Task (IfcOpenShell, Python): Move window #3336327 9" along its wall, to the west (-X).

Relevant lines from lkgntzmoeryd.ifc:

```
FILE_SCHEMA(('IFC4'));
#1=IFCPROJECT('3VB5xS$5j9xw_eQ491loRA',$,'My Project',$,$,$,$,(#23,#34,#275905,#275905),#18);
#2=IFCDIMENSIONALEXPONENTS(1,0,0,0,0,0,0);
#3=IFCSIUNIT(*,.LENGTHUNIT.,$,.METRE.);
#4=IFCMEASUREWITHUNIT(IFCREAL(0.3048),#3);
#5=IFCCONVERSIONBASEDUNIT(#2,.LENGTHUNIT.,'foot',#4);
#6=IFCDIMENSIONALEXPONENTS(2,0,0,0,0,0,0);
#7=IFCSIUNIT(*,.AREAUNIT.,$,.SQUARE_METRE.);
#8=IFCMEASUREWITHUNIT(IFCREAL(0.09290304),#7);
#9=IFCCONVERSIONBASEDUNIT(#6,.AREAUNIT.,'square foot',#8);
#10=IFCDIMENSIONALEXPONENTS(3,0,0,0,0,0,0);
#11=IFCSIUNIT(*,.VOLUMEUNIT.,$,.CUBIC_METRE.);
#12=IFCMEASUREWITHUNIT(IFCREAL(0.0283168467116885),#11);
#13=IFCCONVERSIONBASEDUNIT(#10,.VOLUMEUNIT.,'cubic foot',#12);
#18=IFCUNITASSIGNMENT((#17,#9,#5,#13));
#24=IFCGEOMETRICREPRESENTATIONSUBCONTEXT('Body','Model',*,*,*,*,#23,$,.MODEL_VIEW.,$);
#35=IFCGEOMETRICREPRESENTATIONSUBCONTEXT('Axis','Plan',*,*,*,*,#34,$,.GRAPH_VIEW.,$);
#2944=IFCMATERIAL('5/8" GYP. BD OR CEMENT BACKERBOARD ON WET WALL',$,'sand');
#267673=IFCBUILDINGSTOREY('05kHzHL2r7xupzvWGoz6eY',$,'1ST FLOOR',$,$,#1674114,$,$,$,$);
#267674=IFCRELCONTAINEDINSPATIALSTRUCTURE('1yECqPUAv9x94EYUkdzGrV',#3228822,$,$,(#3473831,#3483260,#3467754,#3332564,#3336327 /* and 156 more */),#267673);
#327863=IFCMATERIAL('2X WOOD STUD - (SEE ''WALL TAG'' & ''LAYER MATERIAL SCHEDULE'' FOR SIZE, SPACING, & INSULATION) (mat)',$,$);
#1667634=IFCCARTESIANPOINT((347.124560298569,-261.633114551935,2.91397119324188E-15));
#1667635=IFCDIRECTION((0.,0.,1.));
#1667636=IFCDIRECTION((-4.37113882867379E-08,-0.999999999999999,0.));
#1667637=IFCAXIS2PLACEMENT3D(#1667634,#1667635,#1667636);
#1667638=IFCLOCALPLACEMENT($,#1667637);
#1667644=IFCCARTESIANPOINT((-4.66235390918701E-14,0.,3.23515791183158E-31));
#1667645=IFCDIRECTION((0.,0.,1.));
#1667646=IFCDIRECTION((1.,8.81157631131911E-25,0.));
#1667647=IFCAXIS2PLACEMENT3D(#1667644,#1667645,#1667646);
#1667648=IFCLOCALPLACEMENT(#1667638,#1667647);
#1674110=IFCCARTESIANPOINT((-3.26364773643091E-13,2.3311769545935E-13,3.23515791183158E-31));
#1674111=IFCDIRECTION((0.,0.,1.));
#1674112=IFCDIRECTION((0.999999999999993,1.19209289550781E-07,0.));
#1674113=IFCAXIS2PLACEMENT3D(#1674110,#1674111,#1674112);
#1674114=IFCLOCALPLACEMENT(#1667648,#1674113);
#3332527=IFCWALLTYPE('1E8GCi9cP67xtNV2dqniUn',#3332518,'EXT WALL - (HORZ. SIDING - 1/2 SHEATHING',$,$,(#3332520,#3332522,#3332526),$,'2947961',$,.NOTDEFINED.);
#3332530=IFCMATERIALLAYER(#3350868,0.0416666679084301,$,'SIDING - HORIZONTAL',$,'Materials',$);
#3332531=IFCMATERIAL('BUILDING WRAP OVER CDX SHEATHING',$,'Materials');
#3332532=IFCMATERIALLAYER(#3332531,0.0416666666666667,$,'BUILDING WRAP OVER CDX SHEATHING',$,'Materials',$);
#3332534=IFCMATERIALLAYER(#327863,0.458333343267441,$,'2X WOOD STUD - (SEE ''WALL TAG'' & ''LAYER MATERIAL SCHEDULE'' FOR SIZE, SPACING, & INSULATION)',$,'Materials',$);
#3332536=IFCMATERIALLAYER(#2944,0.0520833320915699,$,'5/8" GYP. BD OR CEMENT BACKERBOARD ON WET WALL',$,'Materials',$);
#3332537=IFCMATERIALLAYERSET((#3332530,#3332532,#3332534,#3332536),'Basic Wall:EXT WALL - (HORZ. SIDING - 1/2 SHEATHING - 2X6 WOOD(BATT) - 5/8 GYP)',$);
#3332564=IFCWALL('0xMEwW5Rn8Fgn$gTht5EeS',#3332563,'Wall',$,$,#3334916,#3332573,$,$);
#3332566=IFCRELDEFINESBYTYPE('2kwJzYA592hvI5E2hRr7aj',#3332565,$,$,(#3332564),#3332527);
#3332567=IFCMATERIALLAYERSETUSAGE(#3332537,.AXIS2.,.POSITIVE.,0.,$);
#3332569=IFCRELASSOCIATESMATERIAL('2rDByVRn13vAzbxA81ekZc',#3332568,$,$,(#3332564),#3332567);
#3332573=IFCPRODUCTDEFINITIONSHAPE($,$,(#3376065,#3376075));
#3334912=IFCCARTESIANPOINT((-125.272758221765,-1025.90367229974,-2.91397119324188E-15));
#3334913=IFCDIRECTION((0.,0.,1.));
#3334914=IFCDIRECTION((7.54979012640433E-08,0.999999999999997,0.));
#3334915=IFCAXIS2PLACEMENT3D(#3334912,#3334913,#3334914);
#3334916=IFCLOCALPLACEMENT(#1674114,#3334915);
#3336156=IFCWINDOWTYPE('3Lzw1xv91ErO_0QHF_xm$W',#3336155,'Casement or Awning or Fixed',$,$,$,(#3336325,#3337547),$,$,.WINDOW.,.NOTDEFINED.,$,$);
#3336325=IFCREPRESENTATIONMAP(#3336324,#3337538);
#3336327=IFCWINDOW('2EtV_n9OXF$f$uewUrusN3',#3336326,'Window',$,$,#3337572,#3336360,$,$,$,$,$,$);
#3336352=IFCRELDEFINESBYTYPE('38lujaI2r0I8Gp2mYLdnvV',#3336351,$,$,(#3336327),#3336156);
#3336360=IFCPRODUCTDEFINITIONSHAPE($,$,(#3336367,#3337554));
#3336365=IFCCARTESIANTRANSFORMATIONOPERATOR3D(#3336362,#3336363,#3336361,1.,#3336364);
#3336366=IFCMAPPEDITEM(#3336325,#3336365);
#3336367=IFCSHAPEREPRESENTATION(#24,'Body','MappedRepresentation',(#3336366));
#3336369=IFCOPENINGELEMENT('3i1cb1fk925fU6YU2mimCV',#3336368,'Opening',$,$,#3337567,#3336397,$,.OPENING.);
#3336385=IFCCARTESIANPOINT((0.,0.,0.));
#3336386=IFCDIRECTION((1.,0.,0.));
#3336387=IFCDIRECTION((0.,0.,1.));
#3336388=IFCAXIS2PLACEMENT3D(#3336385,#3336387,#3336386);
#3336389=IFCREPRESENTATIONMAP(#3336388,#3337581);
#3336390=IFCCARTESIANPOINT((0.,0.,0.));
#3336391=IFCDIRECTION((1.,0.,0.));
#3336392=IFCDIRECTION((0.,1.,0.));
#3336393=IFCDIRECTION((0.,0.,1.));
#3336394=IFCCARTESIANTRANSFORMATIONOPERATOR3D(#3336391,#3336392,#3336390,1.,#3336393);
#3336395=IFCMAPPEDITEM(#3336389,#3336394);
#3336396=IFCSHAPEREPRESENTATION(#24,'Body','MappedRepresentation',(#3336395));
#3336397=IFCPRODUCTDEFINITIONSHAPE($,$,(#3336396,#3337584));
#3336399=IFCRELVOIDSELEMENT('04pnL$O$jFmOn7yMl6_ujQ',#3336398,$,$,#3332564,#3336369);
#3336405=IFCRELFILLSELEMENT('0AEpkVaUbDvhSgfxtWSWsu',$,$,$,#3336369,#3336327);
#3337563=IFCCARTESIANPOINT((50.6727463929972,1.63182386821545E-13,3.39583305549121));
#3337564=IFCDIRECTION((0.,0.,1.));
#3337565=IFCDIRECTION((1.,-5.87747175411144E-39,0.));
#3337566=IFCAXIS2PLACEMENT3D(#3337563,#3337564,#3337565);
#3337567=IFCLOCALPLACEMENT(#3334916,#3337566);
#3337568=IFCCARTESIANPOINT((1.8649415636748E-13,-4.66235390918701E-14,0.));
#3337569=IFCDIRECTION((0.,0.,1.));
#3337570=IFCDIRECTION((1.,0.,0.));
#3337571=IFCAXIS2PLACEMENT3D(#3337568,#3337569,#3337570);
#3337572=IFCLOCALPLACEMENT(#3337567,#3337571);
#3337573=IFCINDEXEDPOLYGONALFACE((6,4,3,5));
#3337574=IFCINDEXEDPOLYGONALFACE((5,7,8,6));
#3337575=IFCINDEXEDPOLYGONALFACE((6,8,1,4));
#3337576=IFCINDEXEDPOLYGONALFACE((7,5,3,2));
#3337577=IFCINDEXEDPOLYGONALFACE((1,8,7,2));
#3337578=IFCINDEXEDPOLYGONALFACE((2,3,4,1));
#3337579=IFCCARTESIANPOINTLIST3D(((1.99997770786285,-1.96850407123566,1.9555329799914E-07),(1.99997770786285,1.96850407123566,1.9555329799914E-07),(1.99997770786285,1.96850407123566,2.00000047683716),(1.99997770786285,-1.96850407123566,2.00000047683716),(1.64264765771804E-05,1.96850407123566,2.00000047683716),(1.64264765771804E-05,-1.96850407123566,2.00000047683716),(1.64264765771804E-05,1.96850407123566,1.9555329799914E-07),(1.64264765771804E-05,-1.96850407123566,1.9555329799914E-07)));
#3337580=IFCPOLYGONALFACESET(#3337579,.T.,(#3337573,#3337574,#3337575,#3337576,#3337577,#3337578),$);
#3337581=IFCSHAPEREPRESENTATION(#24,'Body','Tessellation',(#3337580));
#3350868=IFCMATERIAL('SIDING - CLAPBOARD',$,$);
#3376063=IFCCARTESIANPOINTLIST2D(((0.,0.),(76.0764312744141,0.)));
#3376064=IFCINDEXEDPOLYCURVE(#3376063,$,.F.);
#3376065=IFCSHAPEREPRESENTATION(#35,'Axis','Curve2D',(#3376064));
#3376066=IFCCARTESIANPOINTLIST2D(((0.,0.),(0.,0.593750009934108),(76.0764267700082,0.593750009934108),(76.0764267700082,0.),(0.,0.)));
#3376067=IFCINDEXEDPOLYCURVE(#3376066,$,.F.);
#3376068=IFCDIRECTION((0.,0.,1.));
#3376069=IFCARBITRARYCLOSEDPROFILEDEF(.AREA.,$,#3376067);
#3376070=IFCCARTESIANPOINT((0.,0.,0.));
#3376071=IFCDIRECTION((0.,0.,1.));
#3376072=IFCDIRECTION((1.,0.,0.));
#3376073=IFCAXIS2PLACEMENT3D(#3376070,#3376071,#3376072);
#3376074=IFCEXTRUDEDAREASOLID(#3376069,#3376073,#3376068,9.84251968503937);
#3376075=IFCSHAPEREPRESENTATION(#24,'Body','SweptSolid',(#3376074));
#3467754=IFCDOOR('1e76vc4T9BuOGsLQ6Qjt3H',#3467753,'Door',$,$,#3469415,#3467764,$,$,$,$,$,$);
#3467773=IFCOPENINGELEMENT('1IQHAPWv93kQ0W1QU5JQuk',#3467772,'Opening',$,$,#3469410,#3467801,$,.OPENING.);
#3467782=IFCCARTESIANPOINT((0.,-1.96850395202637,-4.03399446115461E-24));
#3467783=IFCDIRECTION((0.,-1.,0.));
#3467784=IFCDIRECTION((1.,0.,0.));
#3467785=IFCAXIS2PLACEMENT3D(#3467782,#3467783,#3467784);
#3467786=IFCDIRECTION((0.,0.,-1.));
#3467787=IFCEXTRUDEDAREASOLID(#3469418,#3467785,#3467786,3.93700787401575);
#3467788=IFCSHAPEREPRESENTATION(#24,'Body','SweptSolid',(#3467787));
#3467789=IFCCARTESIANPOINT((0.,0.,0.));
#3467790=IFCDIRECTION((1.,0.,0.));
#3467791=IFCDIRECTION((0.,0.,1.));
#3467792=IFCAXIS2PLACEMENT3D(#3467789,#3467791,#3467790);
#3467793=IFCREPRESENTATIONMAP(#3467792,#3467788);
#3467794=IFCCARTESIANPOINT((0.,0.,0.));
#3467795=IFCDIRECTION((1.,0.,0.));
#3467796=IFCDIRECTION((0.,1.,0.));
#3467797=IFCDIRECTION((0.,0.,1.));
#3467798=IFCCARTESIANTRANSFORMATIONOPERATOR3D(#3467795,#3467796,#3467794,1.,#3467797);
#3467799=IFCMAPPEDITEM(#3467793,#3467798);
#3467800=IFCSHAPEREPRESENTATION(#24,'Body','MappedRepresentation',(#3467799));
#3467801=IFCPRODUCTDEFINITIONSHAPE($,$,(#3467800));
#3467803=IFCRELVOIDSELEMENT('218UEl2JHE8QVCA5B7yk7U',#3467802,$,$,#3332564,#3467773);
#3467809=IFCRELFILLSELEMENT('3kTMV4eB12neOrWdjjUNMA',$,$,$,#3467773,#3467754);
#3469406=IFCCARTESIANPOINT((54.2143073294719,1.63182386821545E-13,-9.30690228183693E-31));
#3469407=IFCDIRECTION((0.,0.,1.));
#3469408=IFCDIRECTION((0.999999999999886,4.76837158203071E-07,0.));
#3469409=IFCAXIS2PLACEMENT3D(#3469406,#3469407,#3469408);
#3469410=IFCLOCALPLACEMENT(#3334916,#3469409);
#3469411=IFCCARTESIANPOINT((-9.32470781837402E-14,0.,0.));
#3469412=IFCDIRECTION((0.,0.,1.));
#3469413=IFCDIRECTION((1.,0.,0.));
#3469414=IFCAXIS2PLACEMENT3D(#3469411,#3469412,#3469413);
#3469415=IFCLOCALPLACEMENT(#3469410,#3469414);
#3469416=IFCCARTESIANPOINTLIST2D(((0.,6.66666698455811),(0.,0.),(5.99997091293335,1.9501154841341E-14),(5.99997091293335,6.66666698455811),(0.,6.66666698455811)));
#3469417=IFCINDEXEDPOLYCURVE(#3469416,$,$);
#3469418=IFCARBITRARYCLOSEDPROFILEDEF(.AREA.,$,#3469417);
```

```python
import ifcopenshell
import ifcopenshell.api.geometry
import ifcopenshell.util.placement
import ifcopenshell.util.unit

model = ifcopenshell.open("lkgntzmoeryd.ifc")
unit_scale = ifcopenshell.util.unit.calculate_unit_scale(model)

window = model.by_guid("2EtV_n9OXF$f$uewUrusN3")
opening = window.FillsVoids[0].RelatingOpeningElement
wall = opening.VoidsElements[0].RelatingBuildingElement

wall_matrix = ifcopenshell.util.placement.get_local_placement(wall.ObjectPlacement)
shift = wall_matrix[:3, 0] * -9 * 0.0254 / unit_scale
before = ifcopenshell.util.placement.get_local_placement(window.ObjectPlacement)[:3, 3].copy()

# The window is placed relative to its opening, so it follows when the opening moves.
matrix = ifcopenshell.util.placement.get_local_placement(opening.ObjectPlacement)
matrix[:3, 3] += shift
ifcopenshell.api.geometry.edit_object_placement(
    model, product=opening, matrix=matrix, is_si=False, should_transform_children=True
)

after = ifcopenshell.util.placement.get_local_placement(window.ObjectPlacement)[:3, 3]
print("window moved by", (after - before).round(3) + 0.0)

model.write("lkgntzmoeryd_v2.ifc")
```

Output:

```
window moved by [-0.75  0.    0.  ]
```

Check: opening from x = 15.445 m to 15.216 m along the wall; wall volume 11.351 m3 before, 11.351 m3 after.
